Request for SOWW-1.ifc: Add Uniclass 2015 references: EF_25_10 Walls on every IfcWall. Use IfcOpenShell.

First a look at what the model holds.

```python
import ifcopenshell

model = ifcopenshell.open("SOWW-1.ifc")
print(model.schema)
print("classifications:", [c.Name for c in model.by_type("IfcClassification")])
for ifc_class in ("IfcDoor", "IfcRoof", "IfcStair", "IfcWall", "IfcWindow"):
    print(ifc_class, len(model.by_type(ifc_class)))
```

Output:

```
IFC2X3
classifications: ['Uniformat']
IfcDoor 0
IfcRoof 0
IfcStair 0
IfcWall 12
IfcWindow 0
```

```python
import ifcopenshell
import ifcopenshell.api.classification

model = ifcopenshell.open("SOWW-1.ifc")

# IFC2X3 requires Source and Edition and has no link from the project to the system.
system = model.create_entity("IfcClassification", Source="NBS", Edition="2015", Name="Uniclass 2015")

codes = {
    "IfcWall": ("EF_25_10", "Walls"),
}
for ifc_class, (code, name) in codes.items():
    products = model.by_type(ifc_class)
    ifcopenshell.api.classification.add_reference(
        model, products=products, classification=system, identification=code, name=name
    )
    print(code, len(products))

model.write("SOWW-1_v2.ifc")
```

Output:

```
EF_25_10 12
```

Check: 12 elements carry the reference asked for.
